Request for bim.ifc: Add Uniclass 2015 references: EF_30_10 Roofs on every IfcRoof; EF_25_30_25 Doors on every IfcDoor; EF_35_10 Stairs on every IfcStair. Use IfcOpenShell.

First a look at what the model holds.

```python
import ifcopenshell

model = ifcopenshell.open("bim.ifc")
print(model.schema)
print("classifications:", [c.Name for c in model.by_type("IfcClassification")])
for ifc_class in ("IfcDoor", "IfcRoof", "IfcStair", "IfcWall", "IfcWindow"):
    print(ifc_class, len(model.by_type(ifc_class)))
```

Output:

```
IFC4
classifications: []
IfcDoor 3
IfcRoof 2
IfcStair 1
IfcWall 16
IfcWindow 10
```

```python
import ifcopenshell
import ifcopenshell.api.classification

model = ifcopenshell.open("bim.ifc")

system = ifcopenshell.api.classification.add_classification(model, classification="Uniclass 2015")

codes = {
    "IfcRoof": ("EF_30_10", "Roofs"),
    "IfcDoor": ("EF_25_30_25", "Doors"),
    "IfcStair": ("EF_35_10", "Stairs"),
}
for ifc_class, (code, name) in codes.items():
    products = model.by_type(ifc_class)
    ifcopenshell.api.classification.add_reference(
        model, products=products, classification=system, identification=code, name=name
    )
    print(code, len(products))

model.write("bim-out.ifc")
```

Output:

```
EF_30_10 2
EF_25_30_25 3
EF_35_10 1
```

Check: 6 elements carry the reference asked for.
